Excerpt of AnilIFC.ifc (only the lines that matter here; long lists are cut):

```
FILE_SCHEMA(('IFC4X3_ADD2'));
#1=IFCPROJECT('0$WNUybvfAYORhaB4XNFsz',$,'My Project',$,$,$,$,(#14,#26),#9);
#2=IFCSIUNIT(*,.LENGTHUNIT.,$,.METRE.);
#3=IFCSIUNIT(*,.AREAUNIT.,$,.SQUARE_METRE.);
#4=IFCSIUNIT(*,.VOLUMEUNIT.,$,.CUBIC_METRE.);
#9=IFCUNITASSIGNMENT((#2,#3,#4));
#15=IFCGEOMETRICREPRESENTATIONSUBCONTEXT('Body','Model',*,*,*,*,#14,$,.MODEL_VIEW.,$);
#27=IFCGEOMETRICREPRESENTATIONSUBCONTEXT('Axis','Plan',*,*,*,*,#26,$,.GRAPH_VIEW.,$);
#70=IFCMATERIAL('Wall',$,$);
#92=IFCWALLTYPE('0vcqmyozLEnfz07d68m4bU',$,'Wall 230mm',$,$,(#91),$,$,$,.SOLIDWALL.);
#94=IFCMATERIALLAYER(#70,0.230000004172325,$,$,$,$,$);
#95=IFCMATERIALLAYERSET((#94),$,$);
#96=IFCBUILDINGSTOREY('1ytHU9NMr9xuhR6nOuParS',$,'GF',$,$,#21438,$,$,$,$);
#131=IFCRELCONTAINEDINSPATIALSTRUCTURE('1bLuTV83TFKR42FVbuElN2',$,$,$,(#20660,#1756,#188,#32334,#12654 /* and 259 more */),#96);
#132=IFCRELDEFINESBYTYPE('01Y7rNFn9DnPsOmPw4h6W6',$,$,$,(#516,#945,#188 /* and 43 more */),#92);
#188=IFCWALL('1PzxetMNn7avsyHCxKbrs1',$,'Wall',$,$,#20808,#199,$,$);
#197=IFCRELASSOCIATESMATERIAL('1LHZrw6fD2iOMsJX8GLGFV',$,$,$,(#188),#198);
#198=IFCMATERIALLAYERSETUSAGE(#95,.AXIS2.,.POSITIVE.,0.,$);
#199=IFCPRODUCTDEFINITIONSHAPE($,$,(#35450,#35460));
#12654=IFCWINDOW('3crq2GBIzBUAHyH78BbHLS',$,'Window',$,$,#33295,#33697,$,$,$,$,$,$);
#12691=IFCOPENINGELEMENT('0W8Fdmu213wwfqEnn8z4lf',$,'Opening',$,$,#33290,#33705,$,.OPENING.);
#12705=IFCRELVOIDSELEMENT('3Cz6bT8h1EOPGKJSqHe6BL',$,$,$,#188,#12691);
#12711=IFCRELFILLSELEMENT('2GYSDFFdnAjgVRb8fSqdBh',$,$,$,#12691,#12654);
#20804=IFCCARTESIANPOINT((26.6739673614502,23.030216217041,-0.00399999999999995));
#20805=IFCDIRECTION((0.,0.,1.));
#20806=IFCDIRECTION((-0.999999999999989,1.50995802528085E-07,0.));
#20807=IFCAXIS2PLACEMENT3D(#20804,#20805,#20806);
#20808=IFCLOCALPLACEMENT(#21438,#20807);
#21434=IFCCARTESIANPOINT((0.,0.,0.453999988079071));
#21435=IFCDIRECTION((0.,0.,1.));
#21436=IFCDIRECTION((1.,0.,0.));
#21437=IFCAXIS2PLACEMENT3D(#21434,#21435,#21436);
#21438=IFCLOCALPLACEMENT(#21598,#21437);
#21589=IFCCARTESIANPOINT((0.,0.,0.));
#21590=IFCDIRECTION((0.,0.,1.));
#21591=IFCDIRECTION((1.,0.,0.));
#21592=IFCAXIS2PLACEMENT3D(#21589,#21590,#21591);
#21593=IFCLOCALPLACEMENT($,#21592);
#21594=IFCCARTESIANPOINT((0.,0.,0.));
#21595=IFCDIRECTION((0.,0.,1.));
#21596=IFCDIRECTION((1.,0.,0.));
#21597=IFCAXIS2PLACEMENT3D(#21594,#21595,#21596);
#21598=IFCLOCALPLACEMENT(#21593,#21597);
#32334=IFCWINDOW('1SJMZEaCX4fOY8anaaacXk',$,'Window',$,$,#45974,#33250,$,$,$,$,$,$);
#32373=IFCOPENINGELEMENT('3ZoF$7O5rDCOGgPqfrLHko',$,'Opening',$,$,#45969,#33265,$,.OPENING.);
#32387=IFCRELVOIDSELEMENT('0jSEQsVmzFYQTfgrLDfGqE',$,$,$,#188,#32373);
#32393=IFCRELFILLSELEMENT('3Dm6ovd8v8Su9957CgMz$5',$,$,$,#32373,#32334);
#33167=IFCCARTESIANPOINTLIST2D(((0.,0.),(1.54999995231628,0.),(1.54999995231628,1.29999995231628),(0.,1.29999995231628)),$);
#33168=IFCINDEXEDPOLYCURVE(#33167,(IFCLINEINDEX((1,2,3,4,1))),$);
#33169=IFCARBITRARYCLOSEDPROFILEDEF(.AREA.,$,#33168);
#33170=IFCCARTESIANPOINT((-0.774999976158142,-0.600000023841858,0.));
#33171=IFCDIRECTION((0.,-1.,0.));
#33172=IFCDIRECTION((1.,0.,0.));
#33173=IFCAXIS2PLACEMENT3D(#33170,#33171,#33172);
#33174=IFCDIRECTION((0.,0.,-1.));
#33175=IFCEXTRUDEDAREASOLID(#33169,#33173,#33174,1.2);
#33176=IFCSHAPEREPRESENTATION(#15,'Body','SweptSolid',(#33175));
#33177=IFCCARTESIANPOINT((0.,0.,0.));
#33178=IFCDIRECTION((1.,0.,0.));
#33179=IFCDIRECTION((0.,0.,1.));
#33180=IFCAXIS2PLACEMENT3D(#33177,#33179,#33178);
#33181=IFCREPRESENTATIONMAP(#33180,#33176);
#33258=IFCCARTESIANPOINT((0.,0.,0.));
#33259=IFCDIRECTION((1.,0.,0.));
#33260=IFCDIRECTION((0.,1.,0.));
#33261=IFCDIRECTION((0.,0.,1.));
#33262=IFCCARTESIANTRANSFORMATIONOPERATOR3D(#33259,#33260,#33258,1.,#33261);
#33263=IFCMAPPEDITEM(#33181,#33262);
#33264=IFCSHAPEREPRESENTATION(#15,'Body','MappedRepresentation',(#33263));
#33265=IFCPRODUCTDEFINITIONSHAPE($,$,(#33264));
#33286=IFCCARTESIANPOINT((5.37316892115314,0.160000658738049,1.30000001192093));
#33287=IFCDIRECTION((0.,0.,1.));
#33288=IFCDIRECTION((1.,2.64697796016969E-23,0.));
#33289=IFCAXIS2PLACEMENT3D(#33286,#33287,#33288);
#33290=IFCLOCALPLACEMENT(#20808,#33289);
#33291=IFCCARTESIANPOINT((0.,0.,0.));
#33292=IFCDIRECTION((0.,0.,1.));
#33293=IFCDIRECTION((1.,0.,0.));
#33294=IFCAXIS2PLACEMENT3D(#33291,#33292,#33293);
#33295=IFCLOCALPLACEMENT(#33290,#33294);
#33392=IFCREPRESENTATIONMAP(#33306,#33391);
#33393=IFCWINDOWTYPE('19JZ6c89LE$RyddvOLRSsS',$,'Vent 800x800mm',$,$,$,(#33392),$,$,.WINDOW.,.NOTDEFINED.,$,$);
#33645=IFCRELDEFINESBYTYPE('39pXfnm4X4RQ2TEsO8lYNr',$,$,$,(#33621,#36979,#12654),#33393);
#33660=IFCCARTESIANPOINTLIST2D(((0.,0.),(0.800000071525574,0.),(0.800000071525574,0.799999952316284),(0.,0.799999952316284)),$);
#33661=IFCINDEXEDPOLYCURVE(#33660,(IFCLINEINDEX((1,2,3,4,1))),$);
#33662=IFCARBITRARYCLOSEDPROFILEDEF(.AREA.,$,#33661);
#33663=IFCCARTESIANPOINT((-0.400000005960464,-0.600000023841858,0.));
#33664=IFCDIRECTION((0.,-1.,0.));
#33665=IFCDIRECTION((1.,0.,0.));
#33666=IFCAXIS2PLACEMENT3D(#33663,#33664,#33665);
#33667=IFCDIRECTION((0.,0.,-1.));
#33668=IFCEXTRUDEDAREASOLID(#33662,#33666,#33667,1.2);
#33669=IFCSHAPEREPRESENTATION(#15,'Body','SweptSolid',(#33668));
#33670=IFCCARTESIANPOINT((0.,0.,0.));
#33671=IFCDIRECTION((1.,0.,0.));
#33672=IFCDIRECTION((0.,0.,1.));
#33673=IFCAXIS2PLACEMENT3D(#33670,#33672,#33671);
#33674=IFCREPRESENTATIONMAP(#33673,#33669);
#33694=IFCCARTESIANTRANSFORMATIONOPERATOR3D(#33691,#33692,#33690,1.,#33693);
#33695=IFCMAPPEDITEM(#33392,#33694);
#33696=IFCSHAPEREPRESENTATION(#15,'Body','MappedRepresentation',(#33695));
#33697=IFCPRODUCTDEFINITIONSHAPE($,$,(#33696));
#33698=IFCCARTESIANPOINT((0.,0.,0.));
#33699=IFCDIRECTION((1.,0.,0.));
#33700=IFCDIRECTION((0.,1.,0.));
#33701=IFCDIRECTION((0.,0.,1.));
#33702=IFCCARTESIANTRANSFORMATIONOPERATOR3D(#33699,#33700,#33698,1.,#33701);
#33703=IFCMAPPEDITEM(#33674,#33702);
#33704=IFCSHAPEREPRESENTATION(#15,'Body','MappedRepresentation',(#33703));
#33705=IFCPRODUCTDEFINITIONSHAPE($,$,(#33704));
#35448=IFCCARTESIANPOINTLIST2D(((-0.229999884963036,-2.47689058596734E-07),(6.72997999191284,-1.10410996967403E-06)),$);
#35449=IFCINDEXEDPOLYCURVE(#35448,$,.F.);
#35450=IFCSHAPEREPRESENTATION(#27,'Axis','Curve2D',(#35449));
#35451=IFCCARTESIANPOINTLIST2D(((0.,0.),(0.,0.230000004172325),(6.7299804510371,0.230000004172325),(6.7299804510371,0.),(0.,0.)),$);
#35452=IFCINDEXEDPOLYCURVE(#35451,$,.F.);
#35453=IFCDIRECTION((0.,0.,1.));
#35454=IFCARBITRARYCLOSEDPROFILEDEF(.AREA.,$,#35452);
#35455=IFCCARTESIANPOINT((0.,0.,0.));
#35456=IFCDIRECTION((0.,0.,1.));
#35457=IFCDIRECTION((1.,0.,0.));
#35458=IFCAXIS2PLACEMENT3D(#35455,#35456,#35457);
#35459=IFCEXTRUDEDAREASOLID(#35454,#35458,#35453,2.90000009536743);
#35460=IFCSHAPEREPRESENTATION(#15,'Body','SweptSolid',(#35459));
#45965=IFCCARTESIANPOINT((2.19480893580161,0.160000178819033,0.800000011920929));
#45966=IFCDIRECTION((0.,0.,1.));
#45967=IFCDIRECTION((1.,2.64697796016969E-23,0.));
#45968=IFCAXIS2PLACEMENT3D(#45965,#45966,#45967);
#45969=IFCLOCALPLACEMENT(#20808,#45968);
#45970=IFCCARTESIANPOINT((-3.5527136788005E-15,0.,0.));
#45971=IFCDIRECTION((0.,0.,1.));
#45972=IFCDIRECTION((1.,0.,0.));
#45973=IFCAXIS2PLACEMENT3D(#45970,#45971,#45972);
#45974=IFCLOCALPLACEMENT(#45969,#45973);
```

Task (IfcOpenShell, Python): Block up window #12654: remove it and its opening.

```python
import ifcopenshell
import ifcopenshell.api.feature
import ifcopenshell.api.root
import ifcopenshell.geom
import ifcopenshell.util.shape

model = ifcopenshell.open("AnilIFC.ifc")
settings = ifcopenshell.geom.settings()


def volume(element):
    """Net volume in cubic metres, openings subtracted."""
    shape = ifcopenshell.geom.create_shape(settings, element)
    return ifcopenshell.util.shape.get_volume(shape.geometry)


window = model.by_guid("3crq2GBIzBUAHyH78BbHLS")
opening = window.FillsVoids[0].RelatingOpeningElement
wall = opening.VoidsElements[0].RelatingBuildingElement
before = volume(wall)

ifcopenshell.api.root.remove_product(model, product=window)
ifcopenshell.api.feature.remove_feature(model, feature=opening)

after = volume(wall)

print(f"wall volume {before:.3f} -> {after:.3f} m3")

model.write("AnilIFC_v2.ifc")
```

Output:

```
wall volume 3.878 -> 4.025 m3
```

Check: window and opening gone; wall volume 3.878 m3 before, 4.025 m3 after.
